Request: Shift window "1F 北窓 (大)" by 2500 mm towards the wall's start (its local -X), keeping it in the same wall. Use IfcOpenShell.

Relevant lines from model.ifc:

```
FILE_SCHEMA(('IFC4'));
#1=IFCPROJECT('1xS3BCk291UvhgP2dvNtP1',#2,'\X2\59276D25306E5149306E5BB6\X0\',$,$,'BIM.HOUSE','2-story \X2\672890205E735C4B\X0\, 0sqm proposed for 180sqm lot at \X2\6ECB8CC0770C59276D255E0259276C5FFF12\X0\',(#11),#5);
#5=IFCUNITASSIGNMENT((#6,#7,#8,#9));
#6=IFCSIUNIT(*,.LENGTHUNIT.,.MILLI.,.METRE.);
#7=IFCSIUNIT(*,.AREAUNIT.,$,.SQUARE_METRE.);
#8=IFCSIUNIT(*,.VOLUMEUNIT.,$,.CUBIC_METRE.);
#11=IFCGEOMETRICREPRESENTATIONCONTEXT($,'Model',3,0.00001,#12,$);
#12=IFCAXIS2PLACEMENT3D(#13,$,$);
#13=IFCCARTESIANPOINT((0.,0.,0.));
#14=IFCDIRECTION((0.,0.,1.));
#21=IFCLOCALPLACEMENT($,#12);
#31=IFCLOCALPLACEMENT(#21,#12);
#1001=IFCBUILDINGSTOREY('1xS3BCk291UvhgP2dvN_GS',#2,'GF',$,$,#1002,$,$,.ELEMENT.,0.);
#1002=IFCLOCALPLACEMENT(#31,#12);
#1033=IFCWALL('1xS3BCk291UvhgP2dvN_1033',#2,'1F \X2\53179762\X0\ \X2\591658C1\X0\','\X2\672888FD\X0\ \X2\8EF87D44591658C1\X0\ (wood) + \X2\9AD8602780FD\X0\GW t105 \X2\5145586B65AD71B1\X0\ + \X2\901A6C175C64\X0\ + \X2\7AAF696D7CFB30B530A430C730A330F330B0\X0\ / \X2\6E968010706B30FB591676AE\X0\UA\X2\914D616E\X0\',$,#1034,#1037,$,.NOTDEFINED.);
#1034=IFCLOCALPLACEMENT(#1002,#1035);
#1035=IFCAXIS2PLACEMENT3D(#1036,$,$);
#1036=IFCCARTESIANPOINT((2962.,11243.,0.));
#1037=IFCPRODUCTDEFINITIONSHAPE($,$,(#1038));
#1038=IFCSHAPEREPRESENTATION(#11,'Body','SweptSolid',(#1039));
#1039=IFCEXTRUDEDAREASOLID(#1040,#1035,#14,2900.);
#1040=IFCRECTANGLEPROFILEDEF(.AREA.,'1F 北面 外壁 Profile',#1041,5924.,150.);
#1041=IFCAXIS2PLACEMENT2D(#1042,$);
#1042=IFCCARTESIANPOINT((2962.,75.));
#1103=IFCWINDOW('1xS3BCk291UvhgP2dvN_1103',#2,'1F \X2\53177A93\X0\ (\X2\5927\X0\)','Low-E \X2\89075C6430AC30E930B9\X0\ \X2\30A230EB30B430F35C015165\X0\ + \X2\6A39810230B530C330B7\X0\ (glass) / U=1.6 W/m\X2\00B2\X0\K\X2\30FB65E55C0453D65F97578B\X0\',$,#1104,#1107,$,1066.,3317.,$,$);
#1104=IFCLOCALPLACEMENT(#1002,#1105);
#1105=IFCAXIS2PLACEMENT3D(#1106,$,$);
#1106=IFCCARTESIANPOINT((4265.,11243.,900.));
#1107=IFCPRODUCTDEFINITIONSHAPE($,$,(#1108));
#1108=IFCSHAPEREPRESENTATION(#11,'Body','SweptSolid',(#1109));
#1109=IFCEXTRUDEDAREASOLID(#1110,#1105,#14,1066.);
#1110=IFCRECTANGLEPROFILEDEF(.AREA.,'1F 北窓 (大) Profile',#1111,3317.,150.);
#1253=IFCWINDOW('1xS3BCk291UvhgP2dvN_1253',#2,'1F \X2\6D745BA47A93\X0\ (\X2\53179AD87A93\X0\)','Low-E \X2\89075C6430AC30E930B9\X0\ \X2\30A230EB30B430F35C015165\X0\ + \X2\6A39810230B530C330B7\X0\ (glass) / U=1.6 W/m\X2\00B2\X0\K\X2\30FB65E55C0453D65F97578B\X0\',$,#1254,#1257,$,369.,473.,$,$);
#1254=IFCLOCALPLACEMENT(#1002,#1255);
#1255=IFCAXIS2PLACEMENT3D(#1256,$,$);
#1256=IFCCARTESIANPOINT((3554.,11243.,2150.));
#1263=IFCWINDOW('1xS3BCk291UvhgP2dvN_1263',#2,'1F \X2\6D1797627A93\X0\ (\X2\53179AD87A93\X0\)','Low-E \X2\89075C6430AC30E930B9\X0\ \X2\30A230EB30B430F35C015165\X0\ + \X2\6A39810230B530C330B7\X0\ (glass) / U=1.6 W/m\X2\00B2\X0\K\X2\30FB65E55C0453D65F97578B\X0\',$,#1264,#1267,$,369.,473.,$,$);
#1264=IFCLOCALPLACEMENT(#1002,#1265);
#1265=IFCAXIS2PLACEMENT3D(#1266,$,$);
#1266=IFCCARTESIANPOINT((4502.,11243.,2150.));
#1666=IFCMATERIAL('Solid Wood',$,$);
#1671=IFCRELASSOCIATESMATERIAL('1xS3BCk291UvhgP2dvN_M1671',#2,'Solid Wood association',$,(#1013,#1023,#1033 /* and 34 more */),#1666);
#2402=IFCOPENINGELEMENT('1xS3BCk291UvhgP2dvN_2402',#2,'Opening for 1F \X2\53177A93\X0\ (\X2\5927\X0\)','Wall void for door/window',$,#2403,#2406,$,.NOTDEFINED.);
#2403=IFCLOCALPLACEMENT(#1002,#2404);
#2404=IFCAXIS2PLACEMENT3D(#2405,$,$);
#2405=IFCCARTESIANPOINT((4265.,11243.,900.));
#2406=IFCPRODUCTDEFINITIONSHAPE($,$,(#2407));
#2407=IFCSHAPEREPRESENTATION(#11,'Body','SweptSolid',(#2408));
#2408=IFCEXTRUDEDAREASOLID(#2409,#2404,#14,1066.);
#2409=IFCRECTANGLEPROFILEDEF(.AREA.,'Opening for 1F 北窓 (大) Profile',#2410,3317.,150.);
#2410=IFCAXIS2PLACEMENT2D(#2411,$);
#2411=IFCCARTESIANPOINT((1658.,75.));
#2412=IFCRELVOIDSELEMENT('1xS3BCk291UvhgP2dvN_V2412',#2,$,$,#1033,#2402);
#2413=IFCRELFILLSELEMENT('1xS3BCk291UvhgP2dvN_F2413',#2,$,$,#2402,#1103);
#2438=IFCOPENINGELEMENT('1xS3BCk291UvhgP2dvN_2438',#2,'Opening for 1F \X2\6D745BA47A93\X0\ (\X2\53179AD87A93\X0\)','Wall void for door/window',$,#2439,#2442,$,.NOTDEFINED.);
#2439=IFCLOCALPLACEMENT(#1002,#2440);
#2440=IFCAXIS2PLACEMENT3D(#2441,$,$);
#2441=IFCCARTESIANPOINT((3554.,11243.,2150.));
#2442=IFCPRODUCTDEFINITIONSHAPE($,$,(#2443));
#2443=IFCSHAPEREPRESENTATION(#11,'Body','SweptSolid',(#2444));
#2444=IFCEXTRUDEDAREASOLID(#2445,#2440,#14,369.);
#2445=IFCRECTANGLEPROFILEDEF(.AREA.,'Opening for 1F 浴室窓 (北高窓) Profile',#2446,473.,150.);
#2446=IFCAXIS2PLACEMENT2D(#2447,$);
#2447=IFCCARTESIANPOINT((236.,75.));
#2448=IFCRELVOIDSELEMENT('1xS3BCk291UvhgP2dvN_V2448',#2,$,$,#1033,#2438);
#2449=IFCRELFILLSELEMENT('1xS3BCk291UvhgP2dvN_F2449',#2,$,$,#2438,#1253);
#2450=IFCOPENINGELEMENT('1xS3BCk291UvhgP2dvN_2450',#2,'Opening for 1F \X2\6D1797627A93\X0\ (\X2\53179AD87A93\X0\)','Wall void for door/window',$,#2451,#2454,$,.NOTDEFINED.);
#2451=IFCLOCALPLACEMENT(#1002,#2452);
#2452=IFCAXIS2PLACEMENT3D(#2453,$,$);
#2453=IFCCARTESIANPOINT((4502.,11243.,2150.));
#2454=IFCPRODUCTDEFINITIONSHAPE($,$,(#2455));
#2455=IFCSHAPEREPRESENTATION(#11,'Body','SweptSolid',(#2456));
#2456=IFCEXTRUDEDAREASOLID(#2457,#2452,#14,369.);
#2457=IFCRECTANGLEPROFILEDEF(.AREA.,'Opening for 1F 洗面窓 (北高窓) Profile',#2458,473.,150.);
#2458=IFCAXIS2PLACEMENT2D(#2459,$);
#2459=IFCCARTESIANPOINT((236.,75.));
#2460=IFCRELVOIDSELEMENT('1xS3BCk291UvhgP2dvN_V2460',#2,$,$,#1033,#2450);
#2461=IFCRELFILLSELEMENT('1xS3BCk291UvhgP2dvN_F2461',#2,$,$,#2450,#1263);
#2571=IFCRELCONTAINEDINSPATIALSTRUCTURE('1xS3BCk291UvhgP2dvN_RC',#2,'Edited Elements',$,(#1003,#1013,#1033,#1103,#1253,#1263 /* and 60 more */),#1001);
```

```python
import ifcopenshell
import ifcopenshell.api.geometry
import ifcopenshell.util.placement

model = ifcopenshell.open("model.ifc")

window = model.by_guid("1xS3BCk291UvhgP2dvN_1103")
opening = window.FillsVoids[0].RelatingOpeningElement
wall = opening.VoidsElements[0].RelatingBuildingElement

wall_matrix = ifcopenshell.util.placement.get_local_placement(wall.ObjectPlacement)
shift = wall_matrix[:3, 0] * -2500.0
before = ifcopenshell.util.placement.get_local_placement(window.ObjectPlacement)[:3, 3].copy()

# The window is not placed relative to its opening, so move both.
for product in (opening, window):
    matrix = ifcopenshell.util.placement.get_local_placement(product.ObjectPlacement)
    matrix[:3, 3] += shift
    ifcopenshell.api.geometry.edit_object_placement(model, product=product, matrix=matrix, is_si=False)

after = ifcopenshell.util.placement.get_local_placement(window.ObjectPlacement)[:3, 3]
print("window moved by", (after - before).round(3) + 0.0)

model.write("model_v2.ifc")
```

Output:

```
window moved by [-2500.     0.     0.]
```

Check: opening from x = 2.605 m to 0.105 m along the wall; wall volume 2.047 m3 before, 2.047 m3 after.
